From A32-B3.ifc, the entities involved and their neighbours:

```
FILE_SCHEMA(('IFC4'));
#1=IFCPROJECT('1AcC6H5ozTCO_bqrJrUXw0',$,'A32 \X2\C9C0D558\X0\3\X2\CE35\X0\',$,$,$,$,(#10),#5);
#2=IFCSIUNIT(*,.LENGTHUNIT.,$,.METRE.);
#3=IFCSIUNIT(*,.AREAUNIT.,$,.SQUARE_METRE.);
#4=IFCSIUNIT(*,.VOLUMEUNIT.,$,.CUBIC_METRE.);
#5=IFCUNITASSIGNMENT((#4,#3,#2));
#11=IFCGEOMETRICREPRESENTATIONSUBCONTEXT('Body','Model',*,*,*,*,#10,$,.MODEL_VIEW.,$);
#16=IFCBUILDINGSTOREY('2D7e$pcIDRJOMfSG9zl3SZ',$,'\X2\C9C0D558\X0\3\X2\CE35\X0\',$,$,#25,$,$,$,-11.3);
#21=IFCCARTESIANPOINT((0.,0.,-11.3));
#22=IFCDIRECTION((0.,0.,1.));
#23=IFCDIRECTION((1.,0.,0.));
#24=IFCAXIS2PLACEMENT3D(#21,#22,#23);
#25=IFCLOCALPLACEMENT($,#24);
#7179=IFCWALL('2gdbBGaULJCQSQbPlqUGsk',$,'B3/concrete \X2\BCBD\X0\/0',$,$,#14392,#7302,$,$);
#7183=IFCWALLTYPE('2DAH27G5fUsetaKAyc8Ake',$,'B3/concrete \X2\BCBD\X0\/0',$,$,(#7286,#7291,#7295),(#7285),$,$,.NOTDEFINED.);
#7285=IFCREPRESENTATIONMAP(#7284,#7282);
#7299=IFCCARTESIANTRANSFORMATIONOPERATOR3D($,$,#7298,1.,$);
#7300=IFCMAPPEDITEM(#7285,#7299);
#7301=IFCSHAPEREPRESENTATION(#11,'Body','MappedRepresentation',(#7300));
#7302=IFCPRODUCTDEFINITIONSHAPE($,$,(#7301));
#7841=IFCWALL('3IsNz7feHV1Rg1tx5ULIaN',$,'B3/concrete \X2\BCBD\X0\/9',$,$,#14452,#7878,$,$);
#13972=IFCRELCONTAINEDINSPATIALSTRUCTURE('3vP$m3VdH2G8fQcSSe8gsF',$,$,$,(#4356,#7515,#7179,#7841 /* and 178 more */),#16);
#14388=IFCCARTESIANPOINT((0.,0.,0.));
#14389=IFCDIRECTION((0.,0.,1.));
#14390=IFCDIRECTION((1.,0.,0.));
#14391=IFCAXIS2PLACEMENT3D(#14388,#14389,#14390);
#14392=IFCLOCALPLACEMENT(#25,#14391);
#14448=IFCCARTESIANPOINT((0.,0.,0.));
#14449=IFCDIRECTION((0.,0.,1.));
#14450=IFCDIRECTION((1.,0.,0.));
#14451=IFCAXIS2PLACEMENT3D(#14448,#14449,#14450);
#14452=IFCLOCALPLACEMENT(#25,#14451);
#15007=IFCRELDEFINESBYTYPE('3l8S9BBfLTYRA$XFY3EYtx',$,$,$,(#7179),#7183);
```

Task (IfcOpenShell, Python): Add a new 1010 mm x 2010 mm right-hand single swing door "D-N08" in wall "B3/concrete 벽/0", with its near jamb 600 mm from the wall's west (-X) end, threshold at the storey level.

```python
import numpy as np
import ifcopenshell
import ifcopenshell.api.feature
import ifcopenshell.api.geometry
import ifcopenshell.api.root
import ifcopenshell.api.spatial
import ifcopenshell.geom
import ifcopenshell.util.element
import ifcopenshell.util.placement
import ifcopenshell.util.representation
import ifcopenshell.util.shape
import ifcopenshell.util.unit

model = ifcopenshell.open("A32-B3.ifc")
unit_scale = ifcopenshell.util.unit.calculate_unit_scale(model)
settings = ifcopenshell.geom.settings()


def volume(element):
    """Net volume in cubic metres, openings subtracted."""
    shape = ifcopenshell.geom.create_shape(settings, element)
    return ifcopenshell.util.shape.get_volume(shape.geometry)


wall = model.by_guid("2gdbBGaULJCQSQbPlqUGsk")
storey = ifcopenshell.util.element.get_container(wall, ifc_class="IfcBuildingStorey")
context = ifcopenshell.util.representation.get_context(model, "Model", "Body", "MODEL_VIEW")
before = volume(wall)

width, height, from_end, sill = 1.01, 2.01, 0.6, 0.0  # metres

# The wall runs along its own X axis, and the end named is its -X end.
wall_shape = ifcopenshell.geom.create_shape(settings, wall)
x, y, z = ifcopenshell.util.shape.get_vertices(wall_shape.geometry).T
start = x.min() + from_end
face, thickness = float(y.min()), float(y.max() - y.min())
wall_matrix = ifcopenshell.util.placement.get_local_placement(wall.ObjectPlacement)
level = ifcopenshell.util.placement.get_local_placement(storey.ObjectPlacement)[2, 3]


def in_wall(x, y):
    """Placement at x, y metres in the wall's axes, at sill height."""
    matrix = wall_matrix.copy()
    matrix[:, 3] = wall_matrix @ np.array([x / unit_scale, y / unit_scale, 0.0, 1.0])
    matrix[2, 3] = level + sill / unit_scale
    return matrix


# Opening: a box that overshoots both wall faces by 50 mm.
opening = ifcopenshell.api.root.create_entity(model, ifc_class="IfcOpeningElement", predefined_type="OPENING")
box = ifcopenshell.api.geometry.add_wall_representation(
    model, context=context, length=width, height=height, thickness=thickness + 0.1
)
ifcopenshell.api.geometry.assign_representation(model, product=opening, representation=box)
ifcopenshell.api.geometry.edit_object_placement(model, product=opening, matrix=in_wall(start, face - 0.05), is_si=False)
ifcopenshell.api.feature.add_feature(model, feature=opening, element=wall)

door = ifcopenshell.api.root.create_entity(model, ifc_class="IfcDoor", name="D-N08", predefined_type="DOOR")
door.OverallWidth, door.OverallHeight = width / unit_scale, height / unit_scale
door.OperationType = "SINGLE_SWING_RIGHT"
body = ifcopenshell.api.geometry.add_door_representation(
    model,
    context=context,
    overall_width=door.OverallWidth,
    overall_height=door.OverallHeight,
    operation_type="SINGLE_SWING_RIGHT",
    lining_properties={"LiningDepth": thickness / unit_scale, "ThresholdDepth": thickness / unit_scale},
)
ifcopenshell.api.geometry.assign_representation(model, product=door, representation=body)
ifcopenshell.api.spatial.assign_container(model, products=[door], relating_structure=storey)
ifcopenshell.api.feature.add_filling(model, opening=opening, element=door)

# The lining spans the wall, so the door starts at the wall face.
ifcopenshell.api.geometry.edit_object_placement(model, product=door, matrix=in_wall(start, face), is_si=False)

after = volume(wall)

print(f"wall volume {before:.3f} -> {after:.3f} m3")

model.write("A32-B3_rev.ifc")
```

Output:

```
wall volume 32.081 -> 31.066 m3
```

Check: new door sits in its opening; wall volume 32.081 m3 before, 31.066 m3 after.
